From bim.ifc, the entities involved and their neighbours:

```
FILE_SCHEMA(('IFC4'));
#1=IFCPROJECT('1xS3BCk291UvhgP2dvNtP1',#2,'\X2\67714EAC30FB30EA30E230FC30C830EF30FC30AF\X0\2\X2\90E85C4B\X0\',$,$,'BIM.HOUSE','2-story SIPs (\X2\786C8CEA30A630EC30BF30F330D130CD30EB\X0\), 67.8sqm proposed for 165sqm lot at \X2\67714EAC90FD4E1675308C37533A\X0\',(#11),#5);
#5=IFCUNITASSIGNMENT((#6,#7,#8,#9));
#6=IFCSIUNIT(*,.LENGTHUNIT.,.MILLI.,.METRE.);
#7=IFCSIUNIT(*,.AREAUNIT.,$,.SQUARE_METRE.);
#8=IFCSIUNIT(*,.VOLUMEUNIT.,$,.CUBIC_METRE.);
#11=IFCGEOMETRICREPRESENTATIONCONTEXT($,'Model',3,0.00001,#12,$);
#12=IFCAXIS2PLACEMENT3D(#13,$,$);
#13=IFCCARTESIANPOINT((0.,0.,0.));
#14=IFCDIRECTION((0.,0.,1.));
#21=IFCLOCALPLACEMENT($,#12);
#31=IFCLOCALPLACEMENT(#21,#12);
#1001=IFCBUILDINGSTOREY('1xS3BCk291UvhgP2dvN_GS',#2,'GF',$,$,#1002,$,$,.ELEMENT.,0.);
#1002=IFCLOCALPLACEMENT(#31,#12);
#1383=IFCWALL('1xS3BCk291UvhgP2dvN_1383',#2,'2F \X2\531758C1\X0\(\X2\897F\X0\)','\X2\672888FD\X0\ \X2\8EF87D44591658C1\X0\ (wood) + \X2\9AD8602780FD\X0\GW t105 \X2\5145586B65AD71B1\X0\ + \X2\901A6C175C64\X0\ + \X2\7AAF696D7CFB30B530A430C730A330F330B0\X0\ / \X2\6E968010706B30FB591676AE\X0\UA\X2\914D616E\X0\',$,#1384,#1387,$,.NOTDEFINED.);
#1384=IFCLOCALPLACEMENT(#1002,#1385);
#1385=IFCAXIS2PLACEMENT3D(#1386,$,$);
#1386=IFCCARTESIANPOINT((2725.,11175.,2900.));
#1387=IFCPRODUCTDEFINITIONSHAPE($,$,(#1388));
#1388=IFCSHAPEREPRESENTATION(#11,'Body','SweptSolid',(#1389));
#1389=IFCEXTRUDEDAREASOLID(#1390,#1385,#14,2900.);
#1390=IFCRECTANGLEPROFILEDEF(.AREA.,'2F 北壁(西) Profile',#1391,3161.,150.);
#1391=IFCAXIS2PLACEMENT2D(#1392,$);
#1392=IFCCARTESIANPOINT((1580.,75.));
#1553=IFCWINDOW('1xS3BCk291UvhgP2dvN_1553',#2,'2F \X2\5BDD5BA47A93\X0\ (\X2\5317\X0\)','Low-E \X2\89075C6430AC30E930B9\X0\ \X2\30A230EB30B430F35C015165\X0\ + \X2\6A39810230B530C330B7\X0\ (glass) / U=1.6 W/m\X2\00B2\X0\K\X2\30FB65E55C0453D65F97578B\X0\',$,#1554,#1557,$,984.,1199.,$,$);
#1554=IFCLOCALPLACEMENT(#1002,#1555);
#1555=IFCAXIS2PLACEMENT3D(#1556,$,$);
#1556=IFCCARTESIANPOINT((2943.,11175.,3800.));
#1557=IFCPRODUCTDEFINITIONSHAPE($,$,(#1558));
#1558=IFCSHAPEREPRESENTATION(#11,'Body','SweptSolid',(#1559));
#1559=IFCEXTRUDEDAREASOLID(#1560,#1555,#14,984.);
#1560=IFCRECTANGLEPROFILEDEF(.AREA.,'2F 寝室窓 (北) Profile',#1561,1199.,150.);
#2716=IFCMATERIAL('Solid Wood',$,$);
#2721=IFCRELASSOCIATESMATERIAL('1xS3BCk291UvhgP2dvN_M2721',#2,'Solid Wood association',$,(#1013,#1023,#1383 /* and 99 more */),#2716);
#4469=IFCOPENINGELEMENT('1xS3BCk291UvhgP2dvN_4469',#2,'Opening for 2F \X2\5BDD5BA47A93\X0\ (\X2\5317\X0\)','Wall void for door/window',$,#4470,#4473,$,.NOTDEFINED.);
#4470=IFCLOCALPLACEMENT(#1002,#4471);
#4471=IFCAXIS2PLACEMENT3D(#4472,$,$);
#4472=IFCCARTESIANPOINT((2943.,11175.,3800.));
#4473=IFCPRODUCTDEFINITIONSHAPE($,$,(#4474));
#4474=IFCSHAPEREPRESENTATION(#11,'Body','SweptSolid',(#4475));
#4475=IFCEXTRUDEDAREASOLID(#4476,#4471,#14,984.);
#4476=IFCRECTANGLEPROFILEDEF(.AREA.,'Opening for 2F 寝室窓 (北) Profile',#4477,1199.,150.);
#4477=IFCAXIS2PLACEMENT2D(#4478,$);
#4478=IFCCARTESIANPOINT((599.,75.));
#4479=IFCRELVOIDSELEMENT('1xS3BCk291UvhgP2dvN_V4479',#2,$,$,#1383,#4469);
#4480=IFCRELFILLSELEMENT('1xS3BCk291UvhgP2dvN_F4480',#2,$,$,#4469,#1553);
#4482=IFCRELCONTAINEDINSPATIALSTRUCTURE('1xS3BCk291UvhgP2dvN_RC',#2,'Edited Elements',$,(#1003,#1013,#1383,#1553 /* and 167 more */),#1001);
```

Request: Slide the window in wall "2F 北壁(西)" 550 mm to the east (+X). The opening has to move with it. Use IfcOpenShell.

```python
import ifcopenshell
import ifcopenshell.api.geometry
import ifcopenshell.util.placement

model = ifcopenshell.open("bim.ifc")

window = model.by_guid("1xS3BCk291UvhgP2dvN_1553")
opening = window.FillsVoids[0].RelatingOpeningElement
wall = opening.VoidsElements[0].RelatingBuildingElement

wall_matrix = ifcopenshell.util.placement.get_local_placement(wall.ObjectPlacement)
shift = wall_matrix[:3, 0] * 550.0
before = ifcopenshell.util.placement.get_local_placement(window.ObjectPlacement)[:3, 3].copy()

# The window is not placed relative to its opening, so move both.
for product in (opening, window):
    matrix = ifcopenshell.util.placement.get_local_placement(product.ObjectPlacement)
    matrix[:3, 3] += shift
    ifcopenshell.api.geometry.edit_object_placement(model, product=product, matrix=matrix, is_si=False)

after = ifcopenshell.util.placement.get_local_placement(window.ObjectPlacement)[:3, 3]
print("window moved by", (after - before).round(3) + 0.0)

model.write("bim_v2.ifc")
```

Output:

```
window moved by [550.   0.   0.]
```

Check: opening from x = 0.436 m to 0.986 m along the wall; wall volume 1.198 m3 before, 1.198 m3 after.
